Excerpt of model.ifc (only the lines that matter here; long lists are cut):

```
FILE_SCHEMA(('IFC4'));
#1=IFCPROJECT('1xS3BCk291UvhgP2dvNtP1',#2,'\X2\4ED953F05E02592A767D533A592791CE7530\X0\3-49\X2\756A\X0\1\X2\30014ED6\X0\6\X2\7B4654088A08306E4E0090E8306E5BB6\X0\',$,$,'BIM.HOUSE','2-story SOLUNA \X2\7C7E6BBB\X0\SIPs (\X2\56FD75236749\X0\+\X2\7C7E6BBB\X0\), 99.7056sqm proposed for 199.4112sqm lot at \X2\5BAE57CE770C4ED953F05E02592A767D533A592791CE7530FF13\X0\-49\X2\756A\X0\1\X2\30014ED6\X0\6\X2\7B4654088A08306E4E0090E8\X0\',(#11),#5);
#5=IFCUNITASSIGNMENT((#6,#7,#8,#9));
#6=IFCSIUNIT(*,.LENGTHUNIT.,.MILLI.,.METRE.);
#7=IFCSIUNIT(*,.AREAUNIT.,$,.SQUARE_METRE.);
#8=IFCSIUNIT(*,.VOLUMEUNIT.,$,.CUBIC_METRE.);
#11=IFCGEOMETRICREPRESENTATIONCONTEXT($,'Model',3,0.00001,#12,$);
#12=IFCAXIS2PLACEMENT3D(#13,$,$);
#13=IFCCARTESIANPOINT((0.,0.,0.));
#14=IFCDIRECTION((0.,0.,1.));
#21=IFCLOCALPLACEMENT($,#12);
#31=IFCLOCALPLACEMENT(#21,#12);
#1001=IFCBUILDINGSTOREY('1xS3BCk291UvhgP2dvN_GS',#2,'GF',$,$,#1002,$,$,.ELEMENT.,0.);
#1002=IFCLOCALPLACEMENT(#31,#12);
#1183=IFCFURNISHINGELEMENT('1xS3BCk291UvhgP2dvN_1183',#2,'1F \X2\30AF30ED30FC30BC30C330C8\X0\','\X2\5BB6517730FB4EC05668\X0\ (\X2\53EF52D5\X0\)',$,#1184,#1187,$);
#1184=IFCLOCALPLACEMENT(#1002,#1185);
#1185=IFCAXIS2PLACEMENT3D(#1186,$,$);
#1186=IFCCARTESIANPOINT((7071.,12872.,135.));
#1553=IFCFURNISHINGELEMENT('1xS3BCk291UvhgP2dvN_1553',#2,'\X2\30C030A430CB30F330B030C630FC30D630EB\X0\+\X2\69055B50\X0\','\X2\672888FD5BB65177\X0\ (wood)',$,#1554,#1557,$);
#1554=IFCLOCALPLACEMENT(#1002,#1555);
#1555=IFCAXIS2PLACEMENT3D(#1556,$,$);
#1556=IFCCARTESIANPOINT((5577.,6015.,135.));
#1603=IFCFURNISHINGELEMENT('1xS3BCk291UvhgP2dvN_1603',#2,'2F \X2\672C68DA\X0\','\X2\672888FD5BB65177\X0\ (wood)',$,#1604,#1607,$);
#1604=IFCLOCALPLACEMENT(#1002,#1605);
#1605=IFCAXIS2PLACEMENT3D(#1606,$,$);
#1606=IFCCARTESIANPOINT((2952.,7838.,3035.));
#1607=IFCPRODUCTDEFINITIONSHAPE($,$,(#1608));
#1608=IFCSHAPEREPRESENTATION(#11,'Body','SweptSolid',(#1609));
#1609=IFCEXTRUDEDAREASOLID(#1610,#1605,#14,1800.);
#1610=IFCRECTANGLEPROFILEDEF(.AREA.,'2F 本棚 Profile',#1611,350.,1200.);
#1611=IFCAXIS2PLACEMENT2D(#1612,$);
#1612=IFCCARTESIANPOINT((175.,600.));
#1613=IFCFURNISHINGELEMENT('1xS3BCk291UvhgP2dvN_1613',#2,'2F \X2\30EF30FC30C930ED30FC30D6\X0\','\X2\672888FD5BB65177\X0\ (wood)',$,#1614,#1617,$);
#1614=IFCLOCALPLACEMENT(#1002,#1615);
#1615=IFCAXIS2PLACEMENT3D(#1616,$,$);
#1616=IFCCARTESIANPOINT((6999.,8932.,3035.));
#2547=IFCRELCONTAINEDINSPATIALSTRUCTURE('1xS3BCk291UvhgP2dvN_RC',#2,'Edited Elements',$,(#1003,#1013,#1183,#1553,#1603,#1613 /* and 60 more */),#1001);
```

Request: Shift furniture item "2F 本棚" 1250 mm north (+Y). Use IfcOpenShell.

```python
import ifcopenshell
import ifcopenshell.api.geometry
import ifcopenshell.util.placement
import ifcopenshell.util.unit

model = ifcopenshell.open("model.ifc")
unit_scale = ifcopenshell.util.unit.calculate_unit_scale(model)

item = model.by_guid("1xS3BCk291UvhgP2dvN_1603")
matrix = ifcopenshell.util.placement.get_local_placement(item.ObjectPlacement)
matrix[1, 3] += 1.25 / unit_scale
ifcopenshell.api.geometry.edit_object_placement(model, product=item, matrix=matrix, is_si=False)

print(ifcopenshell.util.placement.get_local_placement(item.ObjectPlacement).round(3) + 0.0)

model.write("model_rev.ifc")
```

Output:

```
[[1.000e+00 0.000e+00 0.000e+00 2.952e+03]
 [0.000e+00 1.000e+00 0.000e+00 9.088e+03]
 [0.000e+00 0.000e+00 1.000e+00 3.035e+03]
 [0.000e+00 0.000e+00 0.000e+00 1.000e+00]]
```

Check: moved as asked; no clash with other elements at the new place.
